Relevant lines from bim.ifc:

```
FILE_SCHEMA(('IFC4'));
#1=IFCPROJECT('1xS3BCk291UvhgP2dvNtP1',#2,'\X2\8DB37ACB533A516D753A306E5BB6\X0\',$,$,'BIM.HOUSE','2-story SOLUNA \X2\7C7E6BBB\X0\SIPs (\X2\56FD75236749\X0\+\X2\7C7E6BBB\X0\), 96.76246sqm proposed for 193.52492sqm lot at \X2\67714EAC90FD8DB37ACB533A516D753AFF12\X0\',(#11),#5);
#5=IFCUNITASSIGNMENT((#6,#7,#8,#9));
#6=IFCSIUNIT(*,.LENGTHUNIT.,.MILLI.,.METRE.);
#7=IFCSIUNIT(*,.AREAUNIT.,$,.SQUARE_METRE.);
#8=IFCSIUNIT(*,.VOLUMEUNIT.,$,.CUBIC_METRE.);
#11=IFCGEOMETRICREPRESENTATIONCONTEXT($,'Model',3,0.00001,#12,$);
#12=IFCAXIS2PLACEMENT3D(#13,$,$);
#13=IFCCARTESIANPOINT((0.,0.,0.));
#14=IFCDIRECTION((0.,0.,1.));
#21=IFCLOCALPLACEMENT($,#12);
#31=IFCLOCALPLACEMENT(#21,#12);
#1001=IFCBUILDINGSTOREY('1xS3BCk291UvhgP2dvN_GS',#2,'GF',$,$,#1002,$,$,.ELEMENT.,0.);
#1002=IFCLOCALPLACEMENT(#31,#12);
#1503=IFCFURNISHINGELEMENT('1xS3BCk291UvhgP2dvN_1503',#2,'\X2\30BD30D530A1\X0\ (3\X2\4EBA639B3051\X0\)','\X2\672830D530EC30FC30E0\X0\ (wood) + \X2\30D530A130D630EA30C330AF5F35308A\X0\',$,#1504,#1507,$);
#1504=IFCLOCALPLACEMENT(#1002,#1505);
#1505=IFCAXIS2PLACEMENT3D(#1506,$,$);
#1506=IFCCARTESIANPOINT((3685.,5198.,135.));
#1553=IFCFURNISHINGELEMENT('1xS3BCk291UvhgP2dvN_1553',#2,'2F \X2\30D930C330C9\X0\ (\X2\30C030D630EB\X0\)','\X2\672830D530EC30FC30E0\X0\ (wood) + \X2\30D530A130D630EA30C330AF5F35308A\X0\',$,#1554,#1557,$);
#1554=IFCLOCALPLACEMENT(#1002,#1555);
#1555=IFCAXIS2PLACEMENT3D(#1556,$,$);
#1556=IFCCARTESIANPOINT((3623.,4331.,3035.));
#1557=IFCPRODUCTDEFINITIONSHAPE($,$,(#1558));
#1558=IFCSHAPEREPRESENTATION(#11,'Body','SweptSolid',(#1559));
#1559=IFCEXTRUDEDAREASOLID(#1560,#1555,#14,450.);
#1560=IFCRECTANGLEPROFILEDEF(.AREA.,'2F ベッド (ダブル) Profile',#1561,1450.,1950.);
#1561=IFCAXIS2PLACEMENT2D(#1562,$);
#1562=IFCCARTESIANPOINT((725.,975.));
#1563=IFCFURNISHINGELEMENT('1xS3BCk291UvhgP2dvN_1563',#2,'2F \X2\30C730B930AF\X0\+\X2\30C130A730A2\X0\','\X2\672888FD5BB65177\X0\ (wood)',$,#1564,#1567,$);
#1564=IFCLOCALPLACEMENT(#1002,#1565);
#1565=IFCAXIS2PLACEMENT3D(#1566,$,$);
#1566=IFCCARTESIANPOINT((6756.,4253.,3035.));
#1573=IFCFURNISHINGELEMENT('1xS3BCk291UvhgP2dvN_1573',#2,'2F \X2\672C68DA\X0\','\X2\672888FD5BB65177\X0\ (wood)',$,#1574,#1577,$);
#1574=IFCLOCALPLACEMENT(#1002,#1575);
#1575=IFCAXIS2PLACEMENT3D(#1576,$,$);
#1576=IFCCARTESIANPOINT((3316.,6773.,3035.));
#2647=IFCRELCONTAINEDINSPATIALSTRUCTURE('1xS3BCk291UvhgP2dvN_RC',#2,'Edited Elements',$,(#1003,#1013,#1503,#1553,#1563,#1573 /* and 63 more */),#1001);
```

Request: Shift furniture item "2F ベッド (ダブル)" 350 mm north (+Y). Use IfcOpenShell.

```python
import ifcopenshell
import ifcopenshell.api.geometry
import ifcopenshell.util.placement
import ifcopenshell.util.unit

model = ifcopenshell.open("bim.ifc")
unit_scale = ifcopenshell.util.unit.calculate_unit_scale(model)

item = model.by_guid("1xS3BCk291UvhgP2dvN_1553")
matrix = ifcopenshell.util.placement.get_local_placement(item.ObjectPlacement)
matrix[1, 3] += 0.35 / unit_scale
ifcopenshell.api.geometry.edit_object_placement(model, product=item, matrix=matrix, is_si=False)

print(ifcopenshell.util.placement.get_local_placement(item.ObjectPlacement).round(3) + 0.0)

model.write("bim_rev.ifc")
```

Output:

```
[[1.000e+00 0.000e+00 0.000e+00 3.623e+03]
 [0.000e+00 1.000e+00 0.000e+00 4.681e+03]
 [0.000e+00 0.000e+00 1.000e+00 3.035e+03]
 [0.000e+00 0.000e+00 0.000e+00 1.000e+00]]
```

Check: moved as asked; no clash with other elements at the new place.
